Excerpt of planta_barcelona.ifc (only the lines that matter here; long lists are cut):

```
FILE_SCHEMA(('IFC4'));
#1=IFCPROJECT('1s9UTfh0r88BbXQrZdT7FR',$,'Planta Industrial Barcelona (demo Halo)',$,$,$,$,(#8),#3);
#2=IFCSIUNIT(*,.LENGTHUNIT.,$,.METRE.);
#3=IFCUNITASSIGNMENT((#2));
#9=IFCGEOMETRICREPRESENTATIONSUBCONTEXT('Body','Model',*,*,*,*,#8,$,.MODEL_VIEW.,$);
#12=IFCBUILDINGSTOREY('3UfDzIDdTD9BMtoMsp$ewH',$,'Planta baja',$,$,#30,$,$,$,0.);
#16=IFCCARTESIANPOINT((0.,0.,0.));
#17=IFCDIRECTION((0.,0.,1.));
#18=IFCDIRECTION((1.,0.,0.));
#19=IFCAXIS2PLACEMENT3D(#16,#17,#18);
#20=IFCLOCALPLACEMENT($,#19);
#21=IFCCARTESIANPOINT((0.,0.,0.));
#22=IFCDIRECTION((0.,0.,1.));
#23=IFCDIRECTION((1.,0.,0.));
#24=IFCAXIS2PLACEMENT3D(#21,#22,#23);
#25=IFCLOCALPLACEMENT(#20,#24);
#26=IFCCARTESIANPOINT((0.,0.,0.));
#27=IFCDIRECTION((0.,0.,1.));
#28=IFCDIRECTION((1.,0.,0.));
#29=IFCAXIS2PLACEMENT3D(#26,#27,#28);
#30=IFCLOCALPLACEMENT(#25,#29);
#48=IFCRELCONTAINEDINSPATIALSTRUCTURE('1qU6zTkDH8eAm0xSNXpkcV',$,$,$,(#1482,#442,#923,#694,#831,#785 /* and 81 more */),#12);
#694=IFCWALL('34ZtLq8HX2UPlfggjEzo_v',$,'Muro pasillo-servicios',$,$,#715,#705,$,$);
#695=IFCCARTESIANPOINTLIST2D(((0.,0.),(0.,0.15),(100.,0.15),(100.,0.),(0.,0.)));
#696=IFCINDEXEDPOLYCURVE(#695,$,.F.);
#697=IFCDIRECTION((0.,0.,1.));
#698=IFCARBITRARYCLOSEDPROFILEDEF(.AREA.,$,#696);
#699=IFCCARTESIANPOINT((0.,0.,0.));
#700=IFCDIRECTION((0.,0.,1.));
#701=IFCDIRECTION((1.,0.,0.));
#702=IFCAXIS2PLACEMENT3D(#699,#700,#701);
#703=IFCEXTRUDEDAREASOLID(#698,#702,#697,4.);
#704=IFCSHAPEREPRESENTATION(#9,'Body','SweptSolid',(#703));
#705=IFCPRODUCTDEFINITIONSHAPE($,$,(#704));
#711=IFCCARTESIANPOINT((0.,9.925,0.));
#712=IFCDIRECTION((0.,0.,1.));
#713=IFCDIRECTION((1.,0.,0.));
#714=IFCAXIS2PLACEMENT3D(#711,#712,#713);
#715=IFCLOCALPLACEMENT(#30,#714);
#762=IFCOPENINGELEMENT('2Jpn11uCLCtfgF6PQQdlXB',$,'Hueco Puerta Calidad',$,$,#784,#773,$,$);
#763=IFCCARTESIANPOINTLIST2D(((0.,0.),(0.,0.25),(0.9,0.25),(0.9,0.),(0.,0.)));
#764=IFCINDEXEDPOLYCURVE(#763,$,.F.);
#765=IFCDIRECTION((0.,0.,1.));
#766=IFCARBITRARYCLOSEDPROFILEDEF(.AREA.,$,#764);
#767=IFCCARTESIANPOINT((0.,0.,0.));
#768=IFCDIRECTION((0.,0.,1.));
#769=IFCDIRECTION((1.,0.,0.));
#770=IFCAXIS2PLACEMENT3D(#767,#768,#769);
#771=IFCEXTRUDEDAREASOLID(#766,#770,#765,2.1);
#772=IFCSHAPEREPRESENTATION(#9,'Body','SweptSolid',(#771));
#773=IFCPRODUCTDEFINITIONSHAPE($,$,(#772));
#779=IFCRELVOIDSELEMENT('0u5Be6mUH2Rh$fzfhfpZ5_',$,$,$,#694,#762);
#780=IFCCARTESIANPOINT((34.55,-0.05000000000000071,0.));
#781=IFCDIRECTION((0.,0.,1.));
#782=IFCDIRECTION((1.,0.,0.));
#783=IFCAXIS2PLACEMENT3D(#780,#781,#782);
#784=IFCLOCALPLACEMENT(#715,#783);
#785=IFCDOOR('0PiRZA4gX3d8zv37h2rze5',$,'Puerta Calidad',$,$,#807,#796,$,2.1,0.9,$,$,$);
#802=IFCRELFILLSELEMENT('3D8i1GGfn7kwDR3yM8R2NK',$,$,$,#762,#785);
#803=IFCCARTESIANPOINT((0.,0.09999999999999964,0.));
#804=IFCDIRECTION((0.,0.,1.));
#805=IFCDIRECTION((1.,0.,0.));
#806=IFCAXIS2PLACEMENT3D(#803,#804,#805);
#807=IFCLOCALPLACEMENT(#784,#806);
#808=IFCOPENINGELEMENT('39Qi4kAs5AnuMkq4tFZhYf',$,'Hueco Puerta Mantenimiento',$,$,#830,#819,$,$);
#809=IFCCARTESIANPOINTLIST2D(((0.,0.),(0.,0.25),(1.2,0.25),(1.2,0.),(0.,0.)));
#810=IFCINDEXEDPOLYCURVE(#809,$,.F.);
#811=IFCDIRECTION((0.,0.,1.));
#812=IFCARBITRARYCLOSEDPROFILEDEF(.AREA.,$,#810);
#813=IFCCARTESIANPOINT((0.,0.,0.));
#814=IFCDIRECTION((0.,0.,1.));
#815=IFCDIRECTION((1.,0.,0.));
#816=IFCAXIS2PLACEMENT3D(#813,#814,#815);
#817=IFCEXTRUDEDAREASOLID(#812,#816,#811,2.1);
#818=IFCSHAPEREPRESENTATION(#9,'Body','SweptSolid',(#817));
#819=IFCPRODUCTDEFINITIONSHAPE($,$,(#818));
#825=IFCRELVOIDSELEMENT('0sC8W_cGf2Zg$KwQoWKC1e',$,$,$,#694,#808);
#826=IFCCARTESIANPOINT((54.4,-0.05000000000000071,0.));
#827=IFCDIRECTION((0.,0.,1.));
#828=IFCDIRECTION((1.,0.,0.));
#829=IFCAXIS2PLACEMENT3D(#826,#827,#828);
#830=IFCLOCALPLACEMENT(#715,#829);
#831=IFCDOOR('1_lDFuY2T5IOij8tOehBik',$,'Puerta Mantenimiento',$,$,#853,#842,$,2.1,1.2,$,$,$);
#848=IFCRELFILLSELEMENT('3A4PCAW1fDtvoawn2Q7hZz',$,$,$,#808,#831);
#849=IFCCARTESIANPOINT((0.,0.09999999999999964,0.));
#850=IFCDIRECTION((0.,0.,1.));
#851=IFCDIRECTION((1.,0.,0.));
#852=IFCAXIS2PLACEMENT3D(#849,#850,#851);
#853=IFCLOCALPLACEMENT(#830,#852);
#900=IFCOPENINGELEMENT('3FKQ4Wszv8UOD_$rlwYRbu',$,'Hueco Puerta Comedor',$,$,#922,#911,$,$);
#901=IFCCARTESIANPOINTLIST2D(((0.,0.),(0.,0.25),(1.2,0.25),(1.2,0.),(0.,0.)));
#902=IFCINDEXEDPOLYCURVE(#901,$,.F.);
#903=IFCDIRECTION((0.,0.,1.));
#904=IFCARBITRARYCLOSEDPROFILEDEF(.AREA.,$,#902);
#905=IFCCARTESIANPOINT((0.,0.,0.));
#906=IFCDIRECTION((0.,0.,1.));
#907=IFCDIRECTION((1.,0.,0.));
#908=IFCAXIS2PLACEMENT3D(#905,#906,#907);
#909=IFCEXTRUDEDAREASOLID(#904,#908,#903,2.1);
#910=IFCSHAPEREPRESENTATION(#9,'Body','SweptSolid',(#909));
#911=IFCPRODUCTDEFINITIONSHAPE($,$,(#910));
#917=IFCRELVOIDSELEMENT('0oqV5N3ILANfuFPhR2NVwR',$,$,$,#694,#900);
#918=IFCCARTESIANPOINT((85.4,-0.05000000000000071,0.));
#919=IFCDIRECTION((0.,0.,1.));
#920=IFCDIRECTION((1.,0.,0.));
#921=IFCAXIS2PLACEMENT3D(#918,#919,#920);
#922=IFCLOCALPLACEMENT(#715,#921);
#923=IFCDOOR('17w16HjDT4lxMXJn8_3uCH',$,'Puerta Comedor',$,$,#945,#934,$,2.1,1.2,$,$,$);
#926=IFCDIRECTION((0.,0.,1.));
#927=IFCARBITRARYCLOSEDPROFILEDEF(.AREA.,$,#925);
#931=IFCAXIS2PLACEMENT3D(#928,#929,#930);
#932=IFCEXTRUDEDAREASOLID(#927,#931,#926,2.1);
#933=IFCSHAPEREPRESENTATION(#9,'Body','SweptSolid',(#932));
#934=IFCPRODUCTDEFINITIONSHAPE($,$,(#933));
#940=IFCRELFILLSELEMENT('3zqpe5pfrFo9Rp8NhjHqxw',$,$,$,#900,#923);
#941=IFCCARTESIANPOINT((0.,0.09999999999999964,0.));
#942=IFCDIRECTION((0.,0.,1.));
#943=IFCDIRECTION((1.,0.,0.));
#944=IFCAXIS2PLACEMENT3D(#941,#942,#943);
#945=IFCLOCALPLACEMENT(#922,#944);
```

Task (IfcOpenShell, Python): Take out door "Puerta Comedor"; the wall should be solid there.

```python
import ifcopenshell
import ifcopenshell.api.feature
import ifcopenshell.api.root
import ifcopenshell.geom
import ifcopenshell.util.shape

model = ifcopenshell.open("planta_barcelona.ifc")
settings = ifcopenshell.geom.settings()


def volume(element):
    """Net volume in cubic metres, openings subtracted."""
    shape = ifcopenshell.geom.create_shape(settings, element)
    return ifcopenshell.util.shape.get_volume(shape.geometry)


door = model.by_guid("17w16HjDT4lxMXJn8_3uCH")
opening = door.FillsVoids[0].RelatingOpeningElement
wall = opening.VoidsElements[0].RelatingBuildingElement
before = volume(wall)

ifcopenshell.api.root.remove_product(model, product=door)
ifcopenshell.api.feature.remove_feature(model, feature=opening)

after = volume(wall)

print(f"wall volume {before:.3f} -> {after:.3f} m3")

model.write("planta_barcelona_v2.ifc")
```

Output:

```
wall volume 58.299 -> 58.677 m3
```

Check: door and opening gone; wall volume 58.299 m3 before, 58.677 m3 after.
